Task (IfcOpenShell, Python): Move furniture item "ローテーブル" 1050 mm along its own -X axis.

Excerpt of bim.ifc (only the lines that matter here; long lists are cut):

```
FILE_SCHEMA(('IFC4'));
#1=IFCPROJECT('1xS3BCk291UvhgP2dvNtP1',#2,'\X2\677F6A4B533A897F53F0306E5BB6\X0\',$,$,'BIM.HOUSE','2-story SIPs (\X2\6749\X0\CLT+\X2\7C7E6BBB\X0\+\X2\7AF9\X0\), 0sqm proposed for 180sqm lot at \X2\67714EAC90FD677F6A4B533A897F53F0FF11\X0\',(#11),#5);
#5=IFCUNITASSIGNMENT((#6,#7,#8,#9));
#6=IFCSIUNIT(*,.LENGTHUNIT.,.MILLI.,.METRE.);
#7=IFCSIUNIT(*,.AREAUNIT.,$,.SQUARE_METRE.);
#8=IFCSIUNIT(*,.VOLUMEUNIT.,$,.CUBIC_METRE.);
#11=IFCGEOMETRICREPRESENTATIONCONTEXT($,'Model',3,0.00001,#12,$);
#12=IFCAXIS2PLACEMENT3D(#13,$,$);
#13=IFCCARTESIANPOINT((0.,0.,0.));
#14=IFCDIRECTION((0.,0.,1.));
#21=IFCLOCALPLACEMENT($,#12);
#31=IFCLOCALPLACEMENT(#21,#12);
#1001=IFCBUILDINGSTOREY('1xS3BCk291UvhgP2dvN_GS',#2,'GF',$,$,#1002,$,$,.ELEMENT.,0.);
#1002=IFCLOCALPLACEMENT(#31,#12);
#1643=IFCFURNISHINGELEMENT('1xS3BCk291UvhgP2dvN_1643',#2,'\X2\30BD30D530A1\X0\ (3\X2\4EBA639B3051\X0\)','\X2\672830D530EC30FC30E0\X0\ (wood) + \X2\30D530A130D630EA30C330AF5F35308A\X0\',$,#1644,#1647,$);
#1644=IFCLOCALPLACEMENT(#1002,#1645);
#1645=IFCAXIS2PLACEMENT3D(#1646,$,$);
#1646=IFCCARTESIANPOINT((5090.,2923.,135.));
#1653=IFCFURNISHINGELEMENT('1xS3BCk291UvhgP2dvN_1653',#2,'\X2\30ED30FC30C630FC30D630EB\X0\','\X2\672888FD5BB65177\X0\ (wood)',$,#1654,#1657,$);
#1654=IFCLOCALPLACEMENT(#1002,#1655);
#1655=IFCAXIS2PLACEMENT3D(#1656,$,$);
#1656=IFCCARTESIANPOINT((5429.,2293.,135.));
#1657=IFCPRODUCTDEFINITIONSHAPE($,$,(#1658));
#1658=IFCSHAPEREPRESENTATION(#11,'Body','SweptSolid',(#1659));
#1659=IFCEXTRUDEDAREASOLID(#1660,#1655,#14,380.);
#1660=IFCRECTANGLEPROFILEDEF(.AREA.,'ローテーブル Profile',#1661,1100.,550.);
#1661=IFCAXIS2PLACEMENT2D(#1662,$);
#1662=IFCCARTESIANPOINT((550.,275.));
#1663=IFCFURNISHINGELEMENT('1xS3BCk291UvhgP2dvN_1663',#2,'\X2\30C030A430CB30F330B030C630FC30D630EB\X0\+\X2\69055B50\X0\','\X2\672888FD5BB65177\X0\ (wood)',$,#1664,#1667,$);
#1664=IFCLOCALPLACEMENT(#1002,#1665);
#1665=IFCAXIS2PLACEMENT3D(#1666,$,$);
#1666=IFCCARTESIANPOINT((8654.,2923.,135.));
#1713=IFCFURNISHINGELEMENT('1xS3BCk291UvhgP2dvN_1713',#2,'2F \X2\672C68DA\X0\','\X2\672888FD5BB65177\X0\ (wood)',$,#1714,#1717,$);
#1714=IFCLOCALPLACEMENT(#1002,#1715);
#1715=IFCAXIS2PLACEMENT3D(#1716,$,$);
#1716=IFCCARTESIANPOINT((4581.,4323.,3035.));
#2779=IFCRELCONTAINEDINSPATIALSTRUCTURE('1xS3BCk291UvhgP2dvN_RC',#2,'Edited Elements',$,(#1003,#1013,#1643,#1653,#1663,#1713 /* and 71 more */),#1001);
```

```python
import ifcopenshell
import ifcopenshell.api.geometry
import ifcopenshell.util.placement

model = ifcopenshell.open("bim.ifc")

item = model.by_id(1653)
matrix = ifcopenshell.util.placement.get_local_placement(item.ObjectPlacement)
matrix[:3, 3] -= matrix[:3, 0] * 1050.0
ifcopenshell.api.geometry.edit_object_placement(model, product=item, matrix=matrix, is_si=False)

print(ifcopenshell.util.placement.get_local_placement(item.ObjectPlacement).round(3) + 0.0)

model.write("bim_updated.ifc")
```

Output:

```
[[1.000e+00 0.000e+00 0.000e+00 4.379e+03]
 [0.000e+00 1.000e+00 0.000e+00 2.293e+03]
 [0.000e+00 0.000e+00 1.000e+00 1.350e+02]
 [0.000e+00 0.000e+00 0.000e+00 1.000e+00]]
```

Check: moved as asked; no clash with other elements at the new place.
